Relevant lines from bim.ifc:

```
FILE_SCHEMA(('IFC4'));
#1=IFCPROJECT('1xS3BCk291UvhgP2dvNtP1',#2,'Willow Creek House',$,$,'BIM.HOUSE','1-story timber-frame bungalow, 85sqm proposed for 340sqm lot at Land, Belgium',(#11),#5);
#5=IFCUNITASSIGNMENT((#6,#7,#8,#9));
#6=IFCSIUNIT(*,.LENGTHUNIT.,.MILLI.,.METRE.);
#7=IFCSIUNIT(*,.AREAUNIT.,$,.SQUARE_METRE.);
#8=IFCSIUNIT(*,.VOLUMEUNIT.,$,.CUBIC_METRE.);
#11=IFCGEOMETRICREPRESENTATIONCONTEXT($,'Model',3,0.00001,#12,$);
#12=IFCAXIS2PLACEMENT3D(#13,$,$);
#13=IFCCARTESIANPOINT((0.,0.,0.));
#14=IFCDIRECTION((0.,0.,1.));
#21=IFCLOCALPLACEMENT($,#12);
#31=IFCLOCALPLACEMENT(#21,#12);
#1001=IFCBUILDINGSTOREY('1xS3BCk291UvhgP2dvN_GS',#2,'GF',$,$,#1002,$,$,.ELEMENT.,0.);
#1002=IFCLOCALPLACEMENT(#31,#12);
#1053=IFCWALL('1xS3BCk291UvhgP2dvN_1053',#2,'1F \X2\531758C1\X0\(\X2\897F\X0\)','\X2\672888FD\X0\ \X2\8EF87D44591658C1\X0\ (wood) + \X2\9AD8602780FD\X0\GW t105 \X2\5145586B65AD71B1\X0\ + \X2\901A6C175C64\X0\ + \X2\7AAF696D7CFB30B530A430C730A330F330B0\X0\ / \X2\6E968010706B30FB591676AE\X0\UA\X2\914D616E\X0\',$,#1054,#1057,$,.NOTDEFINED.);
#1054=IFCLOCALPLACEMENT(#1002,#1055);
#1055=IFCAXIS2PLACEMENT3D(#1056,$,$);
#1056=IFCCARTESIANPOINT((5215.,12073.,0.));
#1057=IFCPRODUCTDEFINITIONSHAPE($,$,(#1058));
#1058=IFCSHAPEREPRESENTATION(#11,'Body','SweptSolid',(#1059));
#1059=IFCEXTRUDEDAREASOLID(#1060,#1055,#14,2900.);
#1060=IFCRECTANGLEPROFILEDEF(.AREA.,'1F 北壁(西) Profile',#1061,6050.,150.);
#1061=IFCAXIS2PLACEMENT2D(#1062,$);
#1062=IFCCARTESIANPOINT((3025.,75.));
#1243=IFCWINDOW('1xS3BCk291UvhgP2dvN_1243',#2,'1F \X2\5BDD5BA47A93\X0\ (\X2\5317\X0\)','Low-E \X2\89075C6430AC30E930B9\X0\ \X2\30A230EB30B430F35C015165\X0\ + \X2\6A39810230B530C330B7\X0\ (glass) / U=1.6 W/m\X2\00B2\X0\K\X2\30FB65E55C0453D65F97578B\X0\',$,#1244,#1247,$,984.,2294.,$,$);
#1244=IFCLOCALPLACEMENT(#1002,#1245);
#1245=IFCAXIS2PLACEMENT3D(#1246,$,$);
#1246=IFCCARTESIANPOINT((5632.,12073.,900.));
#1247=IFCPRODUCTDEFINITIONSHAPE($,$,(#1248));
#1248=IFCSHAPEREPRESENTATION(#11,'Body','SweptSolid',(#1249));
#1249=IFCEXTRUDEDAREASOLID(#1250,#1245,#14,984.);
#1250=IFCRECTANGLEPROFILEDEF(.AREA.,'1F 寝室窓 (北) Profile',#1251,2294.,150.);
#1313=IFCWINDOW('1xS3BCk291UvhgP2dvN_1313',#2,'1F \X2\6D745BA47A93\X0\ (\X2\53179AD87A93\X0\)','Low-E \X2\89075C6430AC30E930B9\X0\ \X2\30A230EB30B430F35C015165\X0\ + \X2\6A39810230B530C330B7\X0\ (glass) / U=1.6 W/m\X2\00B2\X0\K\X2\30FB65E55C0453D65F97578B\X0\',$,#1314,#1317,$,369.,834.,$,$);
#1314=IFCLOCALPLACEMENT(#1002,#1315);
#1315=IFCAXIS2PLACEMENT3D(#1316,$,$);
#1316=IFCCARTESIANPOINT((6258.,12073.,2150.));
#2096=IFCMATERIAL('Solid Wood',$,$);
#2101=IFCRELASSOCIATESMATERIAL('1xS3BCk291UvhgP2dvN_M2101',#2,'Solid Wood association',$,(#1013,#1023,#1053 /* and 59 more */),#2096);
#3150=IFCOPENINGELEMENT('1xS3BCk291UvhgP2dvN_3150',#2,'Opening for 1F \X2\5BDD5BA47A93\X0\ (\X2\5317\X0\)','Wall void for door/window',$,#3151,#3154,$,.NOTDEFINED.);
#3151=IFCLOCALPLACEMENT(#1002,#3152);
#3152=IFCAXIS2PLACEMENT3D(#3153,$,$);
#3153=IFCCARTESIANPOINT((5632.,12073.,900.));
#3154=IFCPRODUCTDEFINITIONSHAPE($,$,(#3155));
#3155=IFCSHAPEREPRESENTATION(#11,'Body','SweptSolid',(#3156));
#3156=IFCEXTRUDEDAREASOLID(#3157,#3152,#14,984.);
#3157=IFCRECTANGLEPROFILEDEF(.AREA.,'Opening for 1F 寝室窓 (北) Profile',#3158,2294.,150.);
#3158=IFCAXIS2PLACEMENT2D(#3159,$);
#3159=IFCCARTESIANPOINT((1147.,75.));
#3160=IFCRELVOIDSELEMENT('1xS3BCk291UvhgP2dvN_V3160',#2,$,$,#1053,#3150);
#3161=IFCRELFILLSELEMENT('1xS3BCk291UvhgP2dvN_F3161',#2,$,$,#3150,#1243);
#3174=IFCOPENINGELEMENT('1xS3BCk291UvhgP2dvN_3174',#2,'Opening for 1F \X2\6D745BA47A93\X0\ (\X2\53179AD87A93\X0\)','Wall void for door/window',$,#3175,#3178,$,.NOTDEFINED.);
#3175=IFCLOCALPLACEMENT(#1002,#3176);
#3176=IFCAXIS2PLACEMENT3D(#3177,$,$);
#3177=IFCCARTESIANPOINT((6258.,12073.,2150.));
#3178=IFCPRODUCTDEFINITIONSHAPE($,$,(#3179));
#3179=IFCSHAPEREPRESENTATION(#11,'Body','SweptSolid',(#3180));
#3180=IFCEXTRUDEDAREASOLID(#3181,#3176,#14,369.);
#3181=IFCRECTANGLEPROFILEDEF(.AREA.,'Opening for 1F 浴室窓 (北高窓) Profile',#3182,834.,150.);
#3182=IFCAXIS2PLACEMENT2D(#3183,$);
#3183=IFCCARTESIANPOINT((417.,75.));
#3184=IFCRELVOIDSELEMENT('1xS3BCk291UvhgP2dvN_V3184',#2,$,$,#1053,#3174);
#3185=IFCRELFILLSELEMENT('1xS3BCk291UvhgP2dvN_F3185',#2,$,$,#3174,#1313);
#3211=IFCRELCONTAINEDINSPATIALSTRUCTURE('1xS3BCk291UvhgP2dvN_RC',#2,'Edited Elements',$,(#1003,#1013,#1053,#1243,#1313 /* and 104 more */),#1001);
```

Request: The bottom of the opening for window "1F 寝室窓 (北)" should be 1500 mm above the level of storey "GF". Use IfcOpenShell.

```python
import numpy as np
import ifcopenshell
import ifcopenshell.api.geometry
import ifcopenshell.geom
import ifcopenshell.util.element
import ifcopenshell.util.placement
import ifcopenshell.util.shape
import ifcopenshell.util.unit

model = ifcopenshell.open("bim.ifc")
unit_scale = ifcopenshell.util.unit.calculate_unit_scale(model)

window = model.by_id(1243)
opening = window.FillsVoids[0].RelatingOpeningElement
storey = ifcopenshell.util.element.get_container(window, ifc_class="IfcBuildingStorey")
level = ifcopenshell.util.placement.get_local_placement(storey.ObjectPlacement)[2, 3]

# The opening's origin need not be at the sill, so measure its lowest point.
shape = ifcopenshell.geom.create_shape(ifcopenshell.geom.settings(), opening)
bottom = ifcopenshell.util.shape.get_shape_bottom_elevation(shape, shape.geometry) / unit_scale
dz = level + 1.5 / unit_scale - bottom

shift = np.array([0.0, 0.0, dz])
# The window is not placed relative to its opening, so move both.
for product in (opening, window):
    matrix = ifcopenshell.util.placement.get_local_placement(product.ObjectPlacement)
    matrix[:3, 3] += shift
    ifcopenshell.api.geometry.edit_object_placement(model, product=product, matrix=matrix, is_si=False)

print(f"moved by {dz * unit_scale:+.3f} m")

model.write("bim_v2.ifc")
```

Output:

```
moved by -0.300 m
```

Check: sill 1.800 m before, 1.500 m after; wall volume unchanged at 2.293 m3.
